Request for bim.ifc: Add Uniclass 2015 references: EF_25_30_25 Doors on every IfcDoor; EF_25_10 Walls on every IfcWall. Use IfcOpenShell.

First a look at what the model holds.

```python
import ifcopenshell

model = ifcopenshell.open("bim.ifc")
print(model.schema)
print("classifications:", [c.Name for c in model.by_type("IfcClassification")])
for ifc_class in ("IfcDoor", "IfcRoof", "IfcStair", "IfcWall", "IfcWindow"):
    print(ifc_class, len(model.by_type(ifc_class)))
```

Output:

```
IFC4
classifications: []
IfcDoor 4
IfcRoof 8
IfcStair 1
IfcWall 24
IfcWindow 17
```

```python
import ifcopenshell
import ifcopenshell.api.classification

model = ifcopenshell.open("bim.ifc")

system = ifcopenshell.api.classification.add_classification(model, classification="Uniclass 2015")

codes = {
    "IfcDoor": ("EF_25_30_25", "Doors"),
    "IfcWall": ("EF_25_10", "Walls"),
}
for ifc_class, (code, name) in codes.items():
    products = model.by_type(ifc_class)
    ifcopenshell.api.classification.add_reference(
        model, products=products, classification=system, identification=code, name=name
    )
    print(code, len(products))

model.write("bim_updated.ifc")
```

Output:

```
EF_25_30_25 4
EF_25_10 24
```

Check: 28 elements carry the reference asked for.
